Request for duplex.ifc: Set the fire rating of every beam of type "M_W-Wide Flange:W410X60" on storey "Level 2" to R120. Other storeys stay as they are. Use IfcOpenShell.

First a look at what the model holds.

```python
import ifcopenshell
import ifcopenshell.util.element

model = ifcopenshell.open("duplex.ifc")
print(model.schema)
storey = next(s for s in model.by_type("IfcBuildingStorey") if s.Name == "Level 2")
beams = [e for e in ifcopenshell.util.element.get_decomposition(storey) if e.is_a("IfcBeam")]
seen = {}
for e in beams:
    element_type = ifcopenshell.util.element.get_type(e)
    key = (element_type.Name if element_type != e and element_type else None, ifcopenshell.util.element.get_pset(e, "Pset_BeamCommon", "FireRating"))
    seen[key] = seen.get(key, 0) + 1
for (name, value), count in sorted(seen.items(), key=str):
    print(count, "x", name, "|", value)
```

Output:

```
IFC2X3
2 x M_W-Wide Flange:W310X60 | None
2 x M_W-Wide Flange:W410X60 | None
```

```python
import ifcopenshell
import ifcopenshell.api.pset
import ifcopenshell.util.element

model = ifcopenshell.open("duplex.ifc")

storey = next(s for s in model.by_type("IfcBuildingStorey") if s.Name == "Level 2")
beams = [e for e in ifcopenshell.util.element.get_decomposition(storey) if e.is_a("IfcBeam")]

count = 0
for e in beams:
    element_type = ifcopenshell.util.element.get_type(e)
    if element_type in (None, e) or element_type.Name != "M_W-Wide Flange:W410X60":
        continue
    # add_pset returns the element's existing set when there is one.
    pset = ifcopenshell.api.pset.add_pset(model, product=e, name="Pset_BeamCommon")
    ifcopenshell.api.pset.edit_pset(model, pset=pset, properties={"FireRating": "R120"})
    count += 1

print(count, "beams updated")

model.write("duplex_v2.ifc")
```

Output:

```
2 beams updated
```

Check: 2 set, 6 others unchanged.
